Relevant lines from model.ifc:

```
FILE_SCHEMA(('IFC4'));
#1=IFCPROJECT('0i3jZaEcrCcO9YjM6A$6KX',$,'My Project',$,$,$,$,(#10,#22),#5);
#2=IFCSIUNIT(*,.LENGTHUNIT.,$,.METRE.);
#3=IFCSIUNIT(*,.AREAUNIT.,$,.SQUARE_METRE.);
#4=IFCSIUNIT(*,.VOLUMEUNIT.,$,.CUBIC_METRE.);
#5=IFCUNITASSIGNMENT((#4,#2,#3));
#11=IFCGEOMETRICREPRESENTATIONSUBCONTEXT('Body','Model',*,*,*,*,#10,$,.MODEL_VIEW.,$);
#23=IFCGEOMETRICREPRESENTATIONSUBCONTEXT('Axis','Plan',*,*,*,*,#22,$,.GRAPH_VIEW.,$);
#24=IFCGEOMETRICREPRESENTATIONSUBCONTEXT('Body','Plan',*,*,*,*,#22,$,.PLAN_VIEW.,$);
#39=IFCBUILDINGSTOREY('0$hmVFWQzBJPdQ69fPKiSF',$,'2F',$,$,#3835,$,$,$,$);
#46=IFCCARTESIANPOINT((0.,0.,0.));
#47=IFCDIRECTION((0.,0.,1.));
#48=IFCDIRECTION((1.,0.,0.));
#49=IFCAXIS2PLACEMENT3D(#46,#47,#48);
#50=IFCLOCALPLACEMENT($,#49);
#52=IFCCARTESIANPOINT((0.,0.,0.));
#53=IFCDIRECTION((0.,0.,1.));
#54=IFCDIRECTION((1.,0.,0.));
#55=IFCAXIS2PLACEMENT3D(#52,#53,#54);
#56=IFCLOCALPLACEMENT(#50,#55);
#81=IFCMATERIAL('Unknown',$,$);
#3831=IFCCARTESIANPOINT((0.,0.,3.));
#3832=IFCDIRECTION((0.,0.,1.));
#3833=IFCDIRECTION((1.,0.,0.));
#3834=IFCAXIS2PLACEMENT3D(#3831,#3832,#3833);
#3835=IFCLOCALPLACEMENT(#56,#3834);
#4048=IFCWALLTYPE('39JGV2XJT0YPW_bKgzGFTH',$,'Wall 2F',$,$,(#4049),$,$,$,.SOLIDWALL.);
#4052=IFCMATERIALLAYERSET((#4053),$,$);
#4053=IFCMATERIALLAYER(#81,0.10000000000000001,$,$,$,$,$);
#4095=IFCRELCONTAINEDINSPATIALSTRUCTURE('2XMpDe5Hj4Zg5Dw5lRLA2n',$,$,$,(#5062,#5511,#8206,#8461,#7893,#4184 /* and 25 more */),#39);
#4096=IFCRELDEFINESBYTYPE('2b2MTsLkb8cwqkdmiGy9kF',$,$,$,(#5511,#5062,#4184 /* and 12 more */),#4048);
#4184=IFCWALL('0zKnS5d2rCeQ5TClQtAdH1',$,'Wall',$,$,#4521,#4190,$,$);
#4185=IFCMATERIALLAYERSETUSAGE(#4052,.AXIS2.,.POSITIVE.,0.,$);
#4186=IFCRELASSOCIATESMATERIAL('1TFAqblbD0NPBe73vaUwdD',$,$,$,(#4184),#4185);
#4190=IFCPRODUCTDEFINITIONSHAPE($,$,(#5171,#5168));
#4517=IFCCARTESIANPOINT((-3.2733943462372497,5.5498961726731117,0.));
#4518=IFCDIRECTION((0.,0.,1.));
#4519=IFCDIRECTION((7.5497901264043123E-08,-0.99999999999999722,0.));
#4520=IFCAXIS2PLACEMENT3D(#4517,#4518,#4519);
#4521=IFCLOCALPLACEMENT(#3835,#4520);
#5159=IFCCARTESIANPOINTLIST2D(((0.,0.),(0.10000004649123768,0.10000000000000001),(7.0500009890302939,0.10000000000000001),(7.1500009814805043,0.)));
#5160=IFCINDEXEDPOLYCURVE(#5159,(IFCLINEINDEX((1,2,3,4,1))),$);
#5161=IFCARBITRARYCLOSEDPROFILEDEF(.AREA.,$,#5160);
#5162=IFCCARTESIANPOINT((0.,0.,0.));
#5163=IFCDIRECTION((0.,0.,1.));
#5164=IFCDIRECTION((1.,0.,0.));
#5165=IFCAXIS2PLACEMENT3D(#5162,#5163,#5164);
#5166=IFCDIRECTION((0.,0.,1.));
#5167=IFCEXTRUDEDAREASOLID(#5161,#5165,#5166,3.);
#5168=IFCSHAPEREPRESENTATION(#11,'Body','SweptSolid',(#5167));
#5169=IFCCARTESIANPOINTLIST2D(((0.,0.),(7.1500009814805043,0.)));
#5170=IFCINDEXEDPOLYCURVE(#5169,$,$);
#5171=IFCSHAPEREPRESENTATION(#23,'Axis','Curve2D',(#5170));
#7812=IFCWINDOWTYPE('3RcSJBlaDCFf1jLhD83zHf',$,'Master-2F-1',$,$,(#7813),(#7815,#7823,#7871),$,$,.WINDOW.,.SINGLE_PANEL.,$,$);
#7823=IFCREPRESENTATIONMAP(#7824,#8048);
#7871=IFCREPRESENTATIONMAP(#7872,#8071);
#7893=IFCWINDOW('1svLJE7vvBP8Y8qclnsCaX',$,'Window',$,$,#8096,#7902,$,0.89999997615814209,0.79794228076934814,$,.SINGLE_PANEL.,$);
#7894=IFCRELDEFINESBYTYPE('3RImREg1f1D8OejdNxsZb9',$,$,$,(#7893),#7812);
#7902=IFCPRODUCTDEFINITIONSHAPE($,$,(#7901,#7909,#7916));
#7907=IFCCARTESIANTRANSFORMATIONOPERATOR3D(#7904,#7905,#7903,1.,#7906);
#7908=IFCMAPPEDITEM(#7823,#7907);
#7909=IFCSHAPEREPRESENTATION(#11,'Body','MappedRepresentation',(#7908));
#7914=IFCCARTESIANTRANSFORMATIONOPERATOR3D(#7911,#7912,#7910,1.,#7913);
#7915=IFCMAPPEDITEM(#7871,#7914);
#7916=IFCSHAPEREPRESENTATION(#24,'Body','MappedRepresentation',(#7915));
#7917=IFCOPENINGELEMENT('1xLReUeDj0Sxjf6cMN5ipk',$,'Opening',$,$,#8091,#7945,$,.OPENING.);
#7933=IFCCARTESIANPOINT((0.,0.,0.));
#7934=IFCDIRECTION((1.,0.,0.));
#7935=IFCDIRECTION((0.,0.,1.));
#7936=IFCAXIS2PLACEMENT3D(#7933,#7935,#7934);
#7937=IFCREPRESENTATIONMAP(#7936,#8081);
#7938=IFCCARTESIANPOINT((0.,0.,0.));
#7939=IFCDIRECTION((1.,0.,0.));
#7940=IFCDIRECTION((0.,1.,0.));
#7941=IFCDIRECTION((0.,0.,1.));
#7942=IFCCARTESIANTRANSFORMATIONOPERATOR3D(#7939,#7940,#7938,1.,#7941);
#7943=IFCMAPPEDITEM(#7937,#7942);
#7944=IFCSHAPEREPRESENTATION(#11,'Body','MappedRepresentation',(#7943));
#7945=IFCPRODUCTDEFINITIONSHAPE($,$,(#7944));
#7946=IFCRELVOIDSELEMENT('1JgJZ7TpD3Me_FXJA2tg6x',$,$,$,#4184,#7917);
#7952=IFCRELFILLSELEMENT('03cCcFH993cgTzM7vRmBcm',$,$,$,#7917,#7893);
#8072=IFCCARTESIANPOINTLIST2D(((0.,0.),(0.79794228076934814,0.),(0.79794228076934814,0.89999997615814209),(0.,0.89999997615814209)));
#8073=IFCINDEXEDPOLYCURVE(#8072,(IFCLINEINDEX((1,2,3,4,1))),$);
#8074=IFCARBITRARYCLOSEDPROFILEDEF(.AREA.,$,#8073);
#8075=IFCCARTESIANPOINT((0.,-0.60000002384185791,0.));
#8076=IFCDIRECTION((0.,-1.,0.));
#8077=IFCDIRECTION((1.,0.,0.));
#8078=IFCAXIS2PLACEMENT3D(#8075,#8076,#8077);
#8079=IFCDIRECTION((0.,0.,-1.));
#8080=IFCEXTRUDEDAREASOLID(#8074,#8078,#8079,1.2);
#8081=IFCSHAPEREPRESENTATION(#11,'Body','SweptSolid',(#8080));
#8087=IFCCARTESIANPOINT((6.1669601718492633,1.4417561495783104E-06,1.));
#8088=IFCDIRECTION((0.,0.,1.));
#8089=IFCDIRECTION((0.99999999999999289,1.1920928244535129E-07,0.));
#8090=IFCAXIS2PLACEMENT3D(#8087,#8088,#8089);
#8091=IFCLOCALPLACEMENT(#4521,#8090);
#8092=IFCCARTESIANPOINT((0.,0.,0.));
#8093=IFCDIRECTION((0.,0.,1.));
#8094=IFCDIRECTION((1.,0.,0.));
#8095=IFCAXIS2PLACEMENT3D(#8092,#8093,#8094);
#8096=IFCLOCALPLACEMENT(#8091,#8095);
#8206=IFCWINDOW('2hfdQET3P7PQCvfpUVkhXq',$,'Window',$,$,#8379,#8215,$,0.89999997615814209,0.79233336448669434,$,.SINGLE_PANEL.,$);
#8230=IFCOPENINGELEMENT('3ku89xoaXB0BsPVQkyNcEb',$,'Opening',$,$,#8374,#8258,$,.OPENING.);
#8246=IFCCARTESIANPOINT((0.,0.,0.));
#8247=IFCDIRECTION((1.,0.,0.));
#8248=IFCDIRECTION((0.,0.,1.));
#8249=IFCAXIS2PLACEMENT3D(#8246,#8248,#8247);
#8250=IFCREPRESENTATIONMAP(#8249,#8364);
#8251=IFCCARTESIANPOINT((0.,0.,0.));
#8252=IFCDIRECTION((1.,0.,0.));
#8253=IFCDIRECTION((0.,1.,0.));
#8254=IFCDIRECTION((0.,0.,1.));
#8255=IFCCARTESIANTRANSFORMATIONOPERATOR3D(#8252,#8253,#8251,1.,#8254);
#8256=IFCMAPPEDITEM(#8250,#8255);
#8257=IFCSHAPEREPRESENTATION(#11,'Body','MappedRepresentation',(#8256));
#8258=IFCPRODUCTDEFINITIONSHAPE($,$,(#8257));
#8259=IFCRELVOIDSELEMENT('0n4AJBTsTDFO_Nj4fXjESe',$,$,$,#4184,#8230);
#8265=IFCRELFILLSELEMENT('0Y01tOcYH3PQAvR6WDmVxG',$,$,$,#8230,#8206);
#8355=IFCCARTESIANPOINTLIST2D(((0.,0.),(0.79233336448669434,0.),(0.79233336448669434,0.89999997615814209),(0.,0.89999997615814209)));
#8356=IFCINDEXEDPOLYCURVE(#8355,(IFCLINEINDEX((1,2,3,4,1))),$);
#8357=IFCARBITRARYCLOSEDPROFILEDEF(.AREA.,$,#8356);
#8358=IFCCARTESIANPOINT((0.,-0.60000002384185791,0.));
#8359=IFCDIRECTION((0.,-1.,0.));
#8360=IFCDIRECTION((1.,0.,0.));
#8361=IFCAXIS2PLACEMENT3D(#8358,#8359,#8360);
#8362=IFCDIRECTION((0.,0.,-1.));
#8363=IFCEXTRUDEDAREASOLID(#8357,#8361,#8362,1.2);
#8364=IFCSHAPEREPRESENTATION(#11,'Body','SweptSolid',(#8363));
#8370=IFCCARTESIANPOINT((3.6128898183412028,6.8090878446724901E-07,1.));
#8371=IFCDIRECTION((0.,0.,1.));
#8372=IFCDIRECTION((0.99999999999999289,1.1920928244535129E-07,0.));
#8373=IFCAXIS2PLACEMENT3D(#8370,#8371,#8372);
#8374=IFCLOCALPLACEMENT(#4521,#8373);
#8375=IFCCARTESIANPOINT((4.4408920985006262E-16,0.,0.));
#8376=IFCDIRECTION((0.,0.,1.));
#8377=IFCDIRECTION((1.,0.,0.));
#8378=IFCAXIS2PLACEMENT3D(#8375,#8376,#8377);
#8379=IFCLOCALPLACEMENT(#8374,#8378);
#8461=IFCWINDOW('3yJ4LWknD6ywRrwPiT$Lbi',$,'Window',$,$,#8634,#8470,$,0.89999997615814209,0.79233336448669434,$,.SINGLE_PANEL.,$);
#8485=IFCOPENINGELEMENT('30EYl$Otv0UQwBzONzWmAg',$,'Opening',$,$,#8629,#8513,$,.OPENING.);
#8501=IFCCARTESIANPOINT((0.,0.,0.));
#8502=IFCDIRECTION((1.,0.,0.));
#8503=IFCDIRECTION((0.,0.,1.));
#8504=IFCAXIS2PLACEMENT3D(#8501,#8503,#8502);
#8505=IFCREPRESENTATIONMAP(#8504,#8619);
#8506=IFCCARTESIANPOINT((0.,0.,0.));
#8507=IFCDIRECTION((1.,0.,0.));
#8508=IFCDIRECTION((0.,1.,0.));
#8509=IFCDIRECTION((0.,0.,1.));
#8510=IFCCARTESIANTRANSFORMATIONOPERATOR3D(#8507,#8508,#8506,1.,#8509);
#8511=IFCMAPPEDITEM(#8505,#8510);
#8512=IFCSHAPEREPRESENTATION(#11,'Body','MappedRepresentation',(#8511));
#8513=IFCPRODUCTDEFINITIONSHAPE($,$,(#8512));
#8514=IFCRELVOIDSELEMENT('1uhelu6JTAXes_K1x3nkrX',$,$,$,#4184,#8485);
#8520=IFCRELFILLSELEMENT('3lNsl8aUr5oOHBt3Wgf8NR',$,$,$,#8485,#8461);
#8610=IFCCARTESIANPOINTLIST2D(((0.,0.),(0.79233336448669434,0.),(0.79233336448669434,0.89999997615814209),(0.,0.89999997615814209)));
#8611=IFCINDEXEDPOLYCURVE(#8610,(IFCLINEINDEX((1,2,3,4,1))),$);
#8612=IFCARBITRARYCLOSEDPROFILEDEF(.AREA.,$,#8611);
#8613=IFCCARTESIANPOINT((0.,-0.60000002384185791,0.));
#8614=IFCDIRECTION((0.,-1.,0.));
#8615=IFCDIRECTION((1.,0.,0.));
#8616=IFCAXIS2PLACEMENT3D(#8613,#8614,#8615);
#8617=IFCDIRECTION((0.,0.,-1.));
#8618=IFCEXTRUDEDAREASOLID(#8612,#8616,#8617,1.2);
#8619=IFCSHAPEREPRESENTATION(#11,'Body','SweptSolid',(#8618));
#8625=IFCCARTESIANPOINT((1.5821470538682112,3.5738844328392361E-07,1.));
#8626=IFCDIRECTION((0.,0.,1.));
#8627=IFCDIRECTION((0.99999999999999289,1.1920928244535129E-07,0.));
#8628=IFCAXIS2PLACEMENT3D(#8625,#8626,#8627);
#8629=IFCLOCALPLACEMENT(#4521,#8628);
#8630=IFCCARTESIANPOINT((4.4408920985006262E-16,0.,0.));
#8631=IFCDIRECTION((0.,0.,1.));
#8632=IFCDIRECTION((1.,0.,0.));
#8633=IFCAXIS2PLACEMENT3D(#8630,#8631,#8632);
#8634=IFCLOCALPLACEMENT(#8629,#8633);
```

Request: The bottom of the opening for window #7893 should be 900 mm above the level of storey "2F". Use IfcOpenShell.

```python
import numpy as np
import ifcopenshell
import ifcopenshell.api.geometry
import ifcopenshell.geom
import ifcopenshell.util.element
import ifcopenshell.util.placement
import ifcopenshell.util.shape
import ifcopenshell.util.unit

model = ifcopenshell.open("model.ifc")
unit_scale = ifcopenshell.util.unit.calculate_unit_scale(model)

window = model.by_guid("1svLJE7vvBP8Y8qclnsCaX")
opening = window.FillsVoids[0].RelatingOpeningElement
storey = ifcopenshell.util.element.get_container(window, ifc_class="IfcBuildingStorey")
level = ifcopenshell.util.placement.get_local_placement(storey.ObjectPlacement)[2, 3]

# The opening's origin need not be at the sill, so measure its lowest point.
shape = ifcopenshell.geom.create_shape(ifcopenshell.geom.settings(), opening)
bottom = ifcopenshell.util.shape.get_shape_bottom_elevation(shape, shape.geometry) / unit_scale
dz = level + 0.9 / unit_scale - bottom

shift = np.array([0.0, 0.0, dz])
# The window is placed relative to its opening, so it follows when the opening moves.
matrix = ifcopenshell.util.placement.get_local_placement(opening.ObjectPlacement)
matrix[:3, 3] += shift
ifcopenshell.api.geometry.edit_object_placement(
    model, product=opening, matrix=matrix, is_si=False, should_transform_children=True
)

print(f"moved by {dz * unit_scale:+.3f} m")

model.write("model_updated.ifc")
```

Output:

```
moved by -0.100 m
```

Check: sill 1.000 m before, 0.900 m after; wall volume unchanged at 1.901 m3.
